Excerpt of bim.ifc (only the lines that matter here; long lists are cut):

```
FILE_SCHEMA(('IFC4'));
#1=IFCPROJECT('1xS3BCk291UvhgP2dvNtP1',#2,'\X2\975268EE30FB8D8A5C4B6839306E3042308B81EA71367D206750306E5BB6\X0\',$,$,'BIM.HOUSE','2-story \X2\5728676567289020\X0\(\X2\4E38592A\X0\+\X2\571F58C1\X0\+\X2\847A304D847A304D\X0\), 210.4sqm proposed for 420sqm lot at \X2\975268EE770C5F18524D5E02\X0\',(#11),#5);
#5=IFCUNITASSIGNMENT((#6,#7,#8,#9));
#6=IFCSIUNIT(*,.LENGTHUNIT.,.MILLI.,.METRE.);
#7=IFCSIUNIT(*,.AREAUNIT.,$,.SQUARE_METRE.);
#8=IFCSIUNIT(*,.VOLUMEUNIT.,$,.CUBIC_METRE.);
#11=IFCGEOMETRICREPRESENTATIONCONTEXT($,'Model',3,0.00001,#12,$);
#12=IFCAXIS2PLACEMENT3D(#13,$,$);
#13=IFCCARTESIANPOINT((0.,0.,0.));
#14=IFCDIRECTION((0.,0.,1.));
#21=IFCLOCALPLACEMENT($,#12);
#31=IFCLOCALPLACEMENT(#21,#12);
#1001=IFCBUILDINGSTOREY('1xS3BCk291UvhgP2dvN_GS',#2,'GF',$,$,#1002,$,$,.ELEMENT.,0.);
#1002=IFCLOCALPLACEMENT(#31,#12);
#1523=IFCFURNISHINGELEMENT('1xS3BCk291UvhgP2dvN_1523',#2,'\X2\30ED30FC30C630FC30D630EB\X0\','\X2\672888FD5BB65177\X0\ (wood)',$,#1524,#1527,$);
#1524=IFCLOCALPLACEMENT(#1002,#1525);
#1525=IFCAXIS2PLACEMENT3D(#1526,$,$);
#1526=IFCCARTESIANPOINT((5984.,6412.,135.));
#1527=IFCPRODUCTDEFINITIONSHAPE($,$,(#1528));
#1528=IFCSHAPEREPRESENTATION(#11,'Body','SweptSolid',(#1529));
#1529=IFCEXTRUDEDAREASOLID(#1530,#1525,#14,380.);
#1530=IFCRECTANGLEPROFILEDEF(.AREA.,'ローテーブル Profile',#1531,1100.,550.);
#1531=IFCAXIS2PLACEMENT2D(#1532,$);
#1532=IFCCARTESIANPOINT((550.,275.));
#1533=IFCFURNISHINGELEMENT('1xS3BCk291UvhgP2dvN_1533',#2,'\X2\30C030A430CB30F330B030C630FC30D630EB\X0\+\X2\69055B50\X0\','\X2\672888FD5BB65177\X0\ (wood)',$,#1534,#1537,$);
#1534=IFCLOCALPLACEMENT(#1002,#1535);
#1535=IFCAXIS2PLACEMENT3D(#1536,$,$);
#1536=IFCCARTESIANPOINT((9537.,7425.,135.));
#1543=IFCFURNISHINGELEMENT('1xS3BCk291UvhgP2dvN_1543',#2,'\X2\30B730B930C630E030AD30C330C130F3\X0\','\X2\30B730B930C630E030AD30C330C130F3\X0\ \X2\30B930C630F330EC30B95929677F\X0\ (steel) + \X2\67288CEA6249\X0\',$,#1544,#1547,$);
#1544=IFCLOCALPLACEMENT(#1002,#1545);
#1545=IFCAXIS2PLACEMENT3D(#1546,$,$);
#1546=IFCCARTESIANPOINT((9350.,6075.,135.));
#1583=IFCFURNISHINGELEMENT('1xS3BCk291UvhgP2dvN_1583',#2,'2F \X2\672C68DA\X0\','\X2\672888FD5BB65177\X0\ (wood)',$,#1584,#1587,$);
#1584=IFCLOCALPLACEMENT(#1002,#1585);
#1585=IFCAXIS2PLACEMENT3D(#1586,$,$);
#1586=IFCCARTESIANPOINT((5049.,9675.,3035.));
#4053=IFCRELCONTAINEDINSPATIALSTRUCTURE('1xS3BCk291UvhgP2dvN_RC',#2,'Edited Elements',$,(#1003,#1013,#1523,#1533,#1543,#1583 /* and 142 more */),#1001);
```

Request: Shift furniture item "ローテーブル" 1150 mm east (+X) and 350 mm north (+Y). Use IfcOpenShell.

```python
import ifcopenshell
import ifcopenshell.api.geometry
import ifcopenshell.util.placement

model = ifcopenshell.open("bim.ifc")

item = model.by_guid("1xS3BCk291UvhgP2dvN_1523")
matrix = ifcopenshell.util.placement.get_local_placement(item.ObjectPlacement)
matrix[0, 3] += 1150.0
matrix[1, 3] += 350.0
ifcopenshell.api.geometry.edit_object_placement(model, product=item, matrix=matrix, is_si=False)

print(ifcopenshell.util.placement.get_local_placement(item.ObjectPlacement).round(3) + 0.0)

model.write("bim_v2.ifc")
```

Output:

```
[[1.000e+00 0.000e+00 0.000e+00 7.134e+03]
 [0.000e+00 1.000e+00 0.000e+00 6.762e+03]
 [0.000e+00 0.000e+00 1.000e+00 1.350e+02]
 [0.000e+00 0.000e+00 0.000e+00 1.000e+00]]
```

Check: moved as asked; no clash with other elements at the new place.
